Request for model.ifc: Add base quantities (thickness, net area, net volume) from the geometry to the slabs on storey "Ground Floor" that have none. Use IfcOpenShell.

First a look at what the model holds.

```python
import ifcopenshell
import ifcopenshell.util.element
import ifcopenshell.util.unit

model = ifcopenshell.open("model.ifc")
print(model.schema)
for unit_type in ("LENGTHUNIT", "AREAUNIT", "VOLUMEUNIT"):
    print(unit_type, ifcopenshell.util.unit.calculate_unit_scale(model, unit_type))
storey = next(s for s in model.by_type("IfcBuildingStorey") if s.Name == "Ground Floor")
slabs = [e for e in ifcopenshell.util.element.get_decomposition(storey) if e.is_a("IfcSlab")]
for e in sorted(slabs, key=lambda e: e.id()):
    print(e.id(), e.is_a(), e.Name, list(ifcopenshell.util.element.get_psets(e, qtos_only=True)), sep=" | ")
```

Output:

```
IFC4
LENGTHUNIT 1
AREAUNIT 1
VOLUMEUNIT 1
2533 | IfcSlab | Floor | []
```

```python
import ifcopenshell
import ifcopenshell.api.pset
import ifcopenshell.geom
import ifcopenshell.util.element
import ifcopenshell.util.shape
import ifcopenshell.util.unit

model = ifcopenshell.open("model.ifc")
unit_scale = ifcopenshell.util.unit.calculate_unit_scale(model)
area_scale = ifcopenshell.util.unit.calculate_unit_scale(model, "AREAUNIT")
volume_scale = ifcopenshell.util.unit.calculate_unit_scale(model, "VOLUMEUNIT")
settings = ifcopenshell.geom.settings()

storey = next(s for s in model.by_type("IfcBuildingStorey") if s.Name == "Ground Floor")
slabs = [e for e in ifcopenshell.util.element.get_decomposition(storey) if e.is_a("IfcSlab")]

for e in sorted(slabs, key=lambda e: e.id()):
    if ifcopenshell.util.element.get_psets(e, qtos_only=True, should_inherit=False):
        continue
    # Geometry comes back in metres, in the element's own axes.
    shape = ifcopenshell.geom.create_shape(settings, e)
    values = {
        "Width": ifcopenshell.util.shape.get_z(shape.geometry) / unit_scale,
        "NetArea": ifcopenshell.util.shape.get_footprint_area(shape.geometry) / area_scale,
        "NetVolume": ifcopenshell.util.shape.get_volume(shape.geometry) / volume_scale,
    }
    qto = ifcopenshell.api.pset.add_qto(model, product=e, name="Qto_SlabBaseQuantities")
    ifcopenshell.api.pset.edit_qto(model, qto=qto, properties=values)
    print(e.id(), {k: round(v, 3) for k, v in values.items()})

model.write("model_rev.ifc")
```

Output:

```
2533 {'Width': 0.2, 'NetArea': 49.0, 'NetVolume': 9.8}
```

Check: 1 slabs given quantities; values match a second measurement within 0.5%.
